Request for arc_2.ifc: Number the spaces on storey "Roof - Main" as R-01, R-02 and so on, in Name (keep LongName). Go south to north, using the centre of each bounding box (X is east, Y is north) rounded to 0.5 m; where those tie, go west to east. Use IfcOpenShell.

First a look at what the model holds.

```python
import ifcopenshell
import ifcopenshell.util.element
import ifcopenshell.util.placement

model = ifcopenshell.open("arc_2.ifc")
print(model.schema)
storey = next(s for s in model.by_type("IfcBuildingStorey") if s.Name == "Roof - Main")
spaces = [e for e in ifcopenshell.util.element.get_decomposition(storey) if e.is_a("IfcSpace")]
for e in sorted(spaces, key=lambda e: e.id()):
    origin = ifcopenshell.util.placement.get_local_placement(e.ObjectPlacement)[:3, 3]
    print(e.id(), e.Name, e.LongName, origin.round(2) + 0.0, sep=" | ")
```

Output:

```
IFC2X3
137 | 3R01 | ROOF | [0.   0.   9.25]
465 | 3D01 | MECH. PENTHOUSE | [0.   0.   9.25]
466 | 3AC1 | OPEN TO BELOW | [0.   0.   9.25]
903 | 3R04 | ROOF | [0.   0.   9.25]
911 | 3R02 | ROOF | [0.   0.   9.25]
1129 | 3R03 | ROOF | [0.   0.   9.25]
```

```python
import ifcopenshell
import ifcopenshell.geom
import ifcopenshell.util.element
import ifcopenshell.util.shape

model = ifcopenshell.open("arc_2.ifc")
settings = ifcopenshell.geom.settings()
settings.set("use-world-coords", True)


def centre(element):
    shape = ifcopenshell.geom.create_shape(settings, element)
    return ifcopenshell.util.shape.get_bbox_centroid(shape.geometry)


storey = next(s for s in model.by_type("IfcBuildingStorey") if s.Name == "Roof - Main")
spaces = [e for e in ifcopenshell.util.element.get_decomposition(storey) if e.is_a("IfcSpace")]

# Insertion points can sit at a corner or the storey origin, so sort by the geometry (in metres).
centres = {e: centre(e) for e in spaces}
spaces.sort(key=lambda e: (round(centres[e][1] / 0.5), centres[e][0]))

for i, e in enumerate(spaces, start=1):
    number = f"R-{i:02d}"
    e.Name = number
    print(e.id(), number)

model.write("arc_2_rev.ifc")
```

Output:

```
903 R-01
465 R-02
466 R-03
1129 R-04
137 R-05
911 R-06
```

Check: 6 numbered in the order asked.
